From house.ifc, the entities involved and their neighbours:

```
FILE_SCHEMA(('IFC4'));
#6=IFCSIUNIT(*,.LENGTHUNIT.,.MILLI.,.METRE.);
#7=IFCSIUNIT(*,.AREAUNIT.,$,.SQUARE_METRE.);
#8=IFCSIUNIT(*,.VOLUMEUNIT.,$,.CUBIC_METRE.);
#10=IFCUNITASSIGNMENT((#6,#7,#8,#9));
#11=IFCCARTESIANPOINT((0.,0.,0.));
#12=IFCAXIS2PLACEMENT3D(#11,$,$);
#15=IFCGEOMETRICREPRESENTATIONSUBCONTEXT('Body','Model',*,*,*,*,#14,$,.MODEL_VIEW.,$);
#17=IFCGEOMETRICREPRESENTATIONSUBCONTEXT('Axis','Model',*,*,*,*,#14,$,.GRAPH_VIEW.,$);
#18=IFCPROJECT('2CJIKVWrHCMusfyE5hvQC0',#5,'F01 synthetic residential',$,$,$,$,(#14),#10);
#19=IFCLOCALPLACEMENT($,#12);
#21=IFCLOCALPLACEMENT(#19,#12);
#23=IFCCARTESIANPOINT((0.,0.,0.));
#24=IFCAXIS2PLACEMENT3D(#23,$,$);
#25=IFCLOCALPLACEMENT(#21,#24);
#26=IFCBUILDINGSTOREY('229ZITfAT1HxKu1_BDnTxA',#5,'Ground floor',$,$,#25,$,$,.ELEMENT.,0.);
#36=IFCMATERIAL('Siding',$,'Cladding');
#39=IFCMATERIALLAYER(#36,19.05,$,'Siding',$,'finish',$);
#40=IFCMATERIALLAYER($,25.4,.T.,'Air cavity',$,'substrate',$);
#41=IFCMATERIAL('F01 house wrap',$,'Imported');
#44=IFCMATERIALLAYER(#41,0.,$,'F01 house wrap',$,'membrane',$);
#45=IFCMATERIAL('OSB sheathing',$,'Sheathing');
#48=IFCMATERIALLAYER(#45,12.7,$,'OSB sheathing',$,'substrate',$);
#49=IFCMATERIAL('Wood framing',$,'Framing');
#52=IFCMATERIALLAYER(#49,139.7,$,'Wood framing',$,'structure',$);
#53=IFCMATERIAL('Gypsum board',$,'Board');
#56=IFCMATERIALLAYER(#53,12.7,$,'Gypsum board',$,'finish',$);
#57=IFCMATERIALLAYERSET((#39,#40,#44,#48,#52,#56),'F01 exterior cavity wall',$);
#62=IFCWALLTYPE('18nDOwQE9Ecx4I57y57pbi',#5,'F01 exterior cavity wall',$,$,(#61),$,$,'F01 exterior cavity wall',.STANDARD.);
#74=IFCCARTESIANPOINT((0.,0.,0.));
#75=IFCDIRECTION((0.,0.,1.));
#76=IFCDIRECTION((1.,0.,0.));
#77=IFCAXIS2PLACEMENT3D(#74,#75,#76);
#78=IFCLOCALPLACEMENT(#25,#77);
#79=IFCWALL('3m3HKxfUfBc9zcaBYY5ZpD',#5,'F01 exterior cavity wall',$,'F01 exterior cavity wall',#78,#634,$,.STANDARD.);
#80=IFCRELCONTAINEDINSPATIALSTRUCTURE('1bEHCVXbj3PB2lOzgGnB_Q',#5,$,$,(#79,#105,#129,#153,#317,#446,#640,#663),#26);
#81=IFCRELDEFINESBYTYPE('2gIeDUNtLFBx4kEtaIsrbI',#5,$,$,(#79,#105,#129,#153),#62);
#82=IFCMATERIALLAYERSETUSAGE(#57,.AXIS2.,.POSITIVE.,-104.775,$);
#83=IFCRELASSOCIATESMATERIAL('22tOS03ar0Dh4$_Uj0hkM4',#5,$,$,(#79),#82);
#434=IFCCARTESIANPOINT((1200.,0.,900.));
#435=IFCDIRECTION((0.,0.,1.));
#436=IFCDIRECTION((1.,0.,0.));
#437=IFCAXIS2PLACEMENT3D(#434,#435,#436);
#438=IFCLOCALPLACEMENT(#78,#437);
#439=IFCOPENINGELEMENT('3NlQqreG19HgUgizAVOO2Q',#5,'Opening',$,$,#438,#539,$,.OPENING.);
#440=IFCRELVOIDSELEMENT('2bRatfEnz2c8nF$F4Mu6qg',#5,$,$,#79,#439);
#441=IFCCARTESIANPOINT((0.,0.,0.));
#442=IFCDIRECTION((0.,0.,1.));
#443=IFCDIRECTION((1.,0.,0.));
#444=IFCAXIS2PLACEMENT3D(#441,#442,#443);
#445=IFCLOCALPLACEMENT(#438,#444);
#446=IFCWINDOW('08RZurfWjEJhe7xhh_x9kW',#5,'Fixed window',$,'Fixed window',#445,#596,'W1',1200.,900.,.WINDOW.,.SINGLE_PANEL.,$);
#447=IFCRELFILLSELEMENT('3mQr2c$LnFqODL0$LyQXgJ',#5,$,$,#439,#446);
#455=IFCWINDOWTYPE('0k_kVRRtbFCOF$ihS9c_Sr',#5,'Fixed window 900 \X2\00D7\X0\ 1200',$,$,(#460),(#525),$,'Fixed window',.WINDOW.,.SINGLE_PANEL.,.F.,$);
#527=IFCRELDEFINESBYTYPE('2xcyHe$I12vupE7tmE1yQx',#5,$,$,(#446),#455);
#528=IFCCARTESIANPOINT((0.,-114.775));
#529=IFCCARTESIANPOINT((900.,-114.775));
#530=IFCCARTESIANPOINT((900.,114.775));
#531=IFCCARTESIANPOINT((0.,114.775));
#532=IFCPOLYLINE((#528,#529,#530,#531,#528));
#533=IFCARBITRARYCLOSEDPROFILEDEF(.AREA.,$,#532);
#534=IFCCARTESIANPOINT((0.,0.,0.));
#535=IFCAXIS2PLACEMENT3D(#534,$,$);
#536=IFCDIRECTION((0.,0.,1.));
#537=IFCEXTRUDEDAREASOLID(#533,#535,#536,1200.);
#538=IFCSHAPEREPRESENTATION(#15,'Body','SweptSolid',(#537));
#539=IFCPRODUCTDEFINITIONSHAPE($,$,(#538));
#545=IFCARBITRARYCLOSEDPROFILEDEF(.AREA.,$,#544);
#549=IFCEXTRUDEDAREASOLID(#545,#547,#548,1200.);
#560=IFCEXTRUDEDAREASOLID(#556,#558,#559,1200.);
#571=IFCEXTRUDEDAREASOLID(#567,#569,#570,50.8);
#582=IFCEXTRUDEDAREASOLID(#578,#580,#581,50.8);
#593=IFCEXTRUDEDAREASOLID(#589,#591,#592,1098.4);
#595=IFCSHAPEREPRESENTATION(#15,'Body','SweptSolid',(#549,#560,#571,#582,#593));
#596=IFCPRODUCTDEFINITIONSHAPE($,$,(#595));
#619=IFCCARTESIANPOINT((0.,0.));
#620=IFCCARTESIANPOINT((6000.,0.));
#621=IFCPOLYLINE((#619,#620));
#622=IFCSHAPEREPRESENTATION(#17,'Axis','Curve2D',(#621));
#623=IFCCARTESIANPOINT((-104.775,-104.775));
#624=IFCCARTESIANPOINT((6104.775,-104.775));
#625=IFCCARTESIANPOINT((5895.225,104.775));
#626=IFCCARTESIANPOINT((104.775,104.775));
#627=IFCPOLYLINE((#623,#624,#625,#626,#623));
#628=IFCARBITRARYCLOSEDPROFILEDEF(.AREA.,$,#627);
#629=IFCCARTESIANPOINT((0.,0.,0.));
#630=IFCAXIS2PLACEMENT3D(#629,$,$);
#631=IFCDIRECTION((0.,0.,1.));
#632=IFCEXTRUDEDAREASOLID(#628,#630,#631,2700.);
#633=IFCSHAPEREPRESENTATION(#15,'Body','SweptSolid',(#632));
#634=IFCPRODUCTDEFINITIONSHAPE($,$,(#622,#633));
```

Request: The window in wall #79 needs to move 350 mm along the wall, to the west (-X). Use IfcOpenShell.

```python
import ifcopenshell
import ifcopenshell.api.geometry
import ifcopenshell.util.placement
import ifcopenshell.util.unit

model = ifcopenshell.open("house.ifc")
unit_scale = ifcopenshell.util.unit.calculate_unit_scale(model)

window = model.by_id(446)
opening = window.FillsVoids[0].RelatingOpeningElement
wall = opening.VoidsElements[0].RelatingBuildingElement

wall_matrix = ifcopenshell.util.placement.get_local_placement(wall.ObjectPlacement)
shift = wall_matrix[:3, 0] * -0.35 / unit_scale
before = ifcopenshell.util.placement.get_local_placement(window.ObjectPlacement)[:3, 3].copy()

# The window is placed relative to its opening, so it follows when the opening moves.
matrix = ifcopenshell.util.placement.get_local_placement(opening.ObjectPlacement)
matrix[:3, 3] += shift
ifcopenshell.api.geometry.edit_object_placement(
    model, product=opening, matrix=matrix, is_si=False, should_transform_children=True
)

after = ifcopenshell.util.placement.get_local_placement(window.ObjectPlacement)[:3, 3]
print("window moved by", (after - before).round(3) + 0.0)

model.write("house-out.ifc")
```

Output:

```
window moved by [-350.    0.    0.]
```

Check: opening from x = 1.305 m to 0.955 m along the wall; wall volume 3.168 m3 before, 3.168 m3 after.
